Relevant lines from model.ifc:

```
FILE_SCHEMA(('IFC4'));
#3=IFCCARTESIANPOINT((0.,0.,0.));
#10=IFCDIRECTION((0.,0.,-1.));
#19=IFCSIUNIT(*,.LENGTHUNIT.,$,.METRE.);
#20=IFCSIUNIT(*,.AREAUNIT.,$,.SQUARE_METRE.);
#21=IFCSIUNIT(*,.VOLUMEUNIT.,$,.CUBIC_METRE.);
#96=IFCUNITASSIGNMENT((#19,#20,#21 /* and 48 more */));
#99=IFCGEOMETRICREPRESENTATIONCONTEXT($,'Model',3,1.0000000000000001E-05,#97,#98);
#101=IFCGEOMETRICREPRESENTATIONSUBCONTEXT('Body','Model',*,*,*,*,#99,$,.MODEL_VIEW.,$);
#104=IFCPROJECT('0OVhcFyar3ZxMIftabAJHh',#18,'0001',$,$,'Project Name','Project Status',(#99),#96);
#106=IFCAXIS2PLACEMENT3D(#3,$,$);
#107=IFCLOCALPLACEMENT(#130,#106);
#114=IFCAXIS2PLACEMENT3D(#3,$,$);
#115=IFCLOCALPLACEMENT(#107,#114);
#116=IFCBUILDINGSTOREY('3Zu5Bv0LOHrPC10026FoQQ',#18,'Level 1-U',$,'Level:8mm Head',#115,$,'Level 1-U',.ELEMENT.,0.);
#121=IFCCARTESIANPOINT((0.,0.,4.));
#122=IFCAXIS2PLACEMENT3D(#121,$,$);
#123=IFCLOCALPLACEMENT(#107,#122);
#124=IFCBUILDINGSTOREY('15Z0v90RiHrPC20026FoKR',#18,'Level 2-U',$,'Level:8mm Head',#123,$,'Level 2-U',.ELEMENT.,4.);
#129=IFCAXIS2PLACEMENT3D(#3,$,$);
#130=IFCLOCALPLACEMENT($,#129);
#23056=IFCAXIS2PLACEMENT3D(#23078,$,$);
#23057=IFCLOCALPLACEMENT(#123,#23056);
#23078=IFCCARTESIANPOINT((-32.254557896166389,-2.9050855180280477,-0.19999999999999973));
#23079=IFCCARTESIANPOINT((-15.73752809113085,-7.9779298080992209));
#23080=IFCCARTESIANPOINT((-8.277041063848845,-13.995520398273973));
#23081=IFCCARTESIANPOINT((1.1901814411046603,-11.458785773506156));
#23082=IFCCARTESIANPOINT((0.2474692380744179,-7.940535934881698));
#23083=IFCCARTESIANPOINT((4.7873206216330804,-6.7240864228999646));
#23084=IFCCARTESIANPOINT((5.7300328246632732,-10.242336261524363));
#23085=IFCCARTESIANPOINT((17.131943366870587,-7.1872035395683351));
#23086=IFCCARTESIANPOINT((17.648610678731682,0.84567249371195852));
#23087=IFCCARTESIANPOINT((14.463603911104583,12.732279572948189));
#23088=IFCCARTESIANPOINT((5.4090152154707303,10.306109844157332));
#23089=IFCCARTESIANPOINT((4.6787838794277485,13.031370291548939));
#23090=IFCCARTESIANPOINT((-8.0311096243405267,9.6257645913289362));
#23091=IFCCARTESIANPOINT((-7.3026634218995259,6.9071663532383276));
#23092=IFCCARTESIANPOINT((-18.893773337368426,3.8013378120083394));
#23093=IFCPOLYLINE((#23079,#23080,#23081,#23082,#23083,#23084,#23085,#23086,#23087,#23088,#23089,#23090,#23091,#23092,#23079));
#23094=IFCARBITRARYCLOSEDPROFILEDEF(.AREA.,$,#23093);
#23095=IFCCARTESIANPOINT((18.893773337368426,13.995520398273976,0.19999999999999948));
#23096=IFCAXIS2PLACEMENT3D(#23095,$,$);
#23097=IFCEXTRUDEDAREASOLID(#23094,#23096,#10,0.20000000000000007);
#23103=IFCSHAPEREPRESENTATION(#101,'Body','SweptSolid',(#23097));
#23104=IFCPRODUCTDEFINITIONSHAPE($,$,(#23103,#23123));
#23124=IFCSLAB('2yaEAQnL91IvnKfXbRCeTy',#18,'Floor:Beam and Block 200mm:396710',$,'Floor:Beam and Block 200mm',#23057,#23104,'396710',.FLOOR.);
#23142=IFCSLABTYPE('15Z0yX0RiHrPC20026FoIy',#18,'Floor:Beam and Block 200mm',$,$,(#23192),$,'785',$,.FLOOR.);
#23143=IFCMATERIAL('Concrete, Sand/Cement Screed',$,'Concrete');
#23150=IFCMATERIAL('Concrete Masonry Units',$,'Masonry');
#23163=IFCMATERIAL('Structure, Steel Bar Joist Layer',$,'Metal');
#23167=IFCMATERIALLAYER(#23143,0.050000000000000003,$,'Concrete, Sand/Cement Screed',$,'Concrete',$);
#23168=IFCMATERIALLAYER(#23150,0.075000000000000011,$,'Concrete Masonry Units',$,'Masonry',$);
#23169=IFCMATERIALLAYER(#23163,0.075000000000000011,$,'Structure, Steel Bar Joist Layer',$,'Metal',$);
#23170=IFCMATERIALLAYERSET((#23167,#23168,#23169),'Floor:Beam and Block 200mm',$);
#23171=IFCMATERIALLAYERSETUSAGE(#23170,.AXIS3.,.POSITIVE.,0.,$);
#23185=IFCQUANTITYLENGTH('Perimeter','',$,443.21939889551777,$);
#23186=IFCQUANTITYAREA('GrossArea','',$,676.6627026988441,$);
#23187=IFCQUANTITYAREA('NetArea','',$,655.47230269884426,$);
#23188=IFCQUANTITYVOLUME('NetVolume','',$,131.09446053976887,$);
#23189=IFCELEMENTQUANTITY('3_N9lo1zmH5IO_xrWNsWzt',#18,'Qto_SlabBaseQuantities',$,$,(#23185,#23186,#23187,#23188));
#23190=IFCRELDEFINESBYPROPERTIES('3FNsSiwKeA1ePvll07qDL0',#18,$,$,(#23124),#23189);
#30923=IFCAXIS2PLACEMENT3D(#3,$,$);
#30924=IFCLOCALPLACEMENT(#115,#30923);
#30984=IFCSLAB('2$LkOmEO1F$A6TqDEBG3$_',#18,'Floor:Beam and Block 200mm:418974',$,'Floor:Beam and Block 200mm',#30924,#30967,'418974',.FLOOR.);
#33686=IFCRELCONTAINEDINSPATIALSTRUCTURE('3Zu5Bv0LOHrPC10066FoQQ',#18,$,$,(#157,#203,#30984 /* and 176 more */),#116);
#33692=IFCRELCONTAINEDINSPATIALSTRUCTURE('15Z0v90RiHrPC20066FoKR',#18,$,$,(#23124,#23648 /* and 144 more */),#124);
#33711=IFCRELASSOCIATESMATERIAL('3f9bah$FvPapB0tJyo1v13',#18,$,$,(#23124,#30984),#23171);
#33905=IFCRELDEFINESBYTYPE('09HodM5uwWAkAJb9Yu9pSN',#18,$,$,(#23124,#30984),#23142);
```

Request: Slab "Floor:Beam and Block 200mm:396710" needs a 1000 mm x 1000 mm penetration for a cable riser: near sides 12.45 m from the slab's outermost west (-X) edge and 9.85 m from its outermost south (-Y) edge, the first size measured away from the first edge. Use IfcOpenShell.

```python
import numpy as np
import ifcopenshell
import ifcopenshell.api.feature
import ifcopenshell.api.geometry
import ifcopenshell.api.pset
import ifcopenshell.api.root
import ifcopenshell.geom
import ifcopenshell.util.element
import ifcopenshell.util.placement
import ifcopenshell.util.representation
import ifcopenshell.util.shape
import ifcopenshell.util.unit

model = ifcopenshell.open("model.ifc")
unit_scale = ifcopenshell.util.unit.calculate_unit_scale(model)
area_scale = ifcopenshell.util.unit.calculate_unit_scale(model, "AREAUNIT")
volume_scale = ifcopenshell.util.unit.calculate_unit_scale(model, "VOLUMEUNIT")
settings = ifcopenshell.geom.settings()


def volume(element):
    """Net volume in cubic metres, openings subtracted."""
    shape = ifcopenshell.geom.create_shape(settings, element)
    return ifcopenshell.util.shape.get_volume(shape.geometry)


slab = model.by_id(23124)
before = volume(slab)

# Extent in the slab's own axes, in metres. The edges named are its -X and -Y sides.
slab_shape = ifcopenshell.geom.create_shape(settings, slab)
vertices = ifcopenshell.util.shape.get_vertices(slab_shape.geometry)
x_min, y_min, bottom = vertices.min(axis=0)
top = vertices[:, 2].max()

opening = ifcopenshell.api.root.create_entity(model, ifc_class="IfcOpeningElement", name="Cable riser opening", predefined_type="OPENING")
context = ifcopenshell.util.representation.get_context(model, "Model", "Body", "MODEL_VIEW")
width, depth = 1, 1
outline = [(0.0, 0.0), (width, 0.0), (width, depth), (0.0, depth), (0.0, 0.0)]
# Overshoot both faces by 50 mm so the cut is clean.
shape = ifcopenshell.api.geometry.add_slab_representation(
    model, context=context, depth=top - bottom + 0.1, polyline=outline
)
ifcopenshell.api.geometry.assign_representation(model, product=opening, representation=shape)

matrix = ifcopenshell.util.placement.get_local_placement(slab.ObjectPlacement)
matrix[:, 3] = matrix @ np.append(np.array([x_min + 12.45, y_min + 9.85, bottom - 0.05]) / unit_scale, 1.0)
ifcopenshell.api.geometry.edit_object_placement(model, product=opening, matrix=matrix, is_si=False)
ifcopenshell.api.feature.add_feature(model, feature=opening, element=slab)

after = volume(slab)

# Update the slab's stored quantities.
qto = model.by_id(ifcopenshell.util.element.get_pset(slab, "Qto_SlabBaseQuantities", should_inherit=False)["id"])
ifcopenshell.api.pset.edit_qto(model, qto=qto, properties={
    "NetArea": after / (top - bottom) / area_scale,
    "NetVolume": after / volume_scale,
})

print(f"slab volume {before:.3f} -> {after:.3f} m3")

model.write("model-out.ifc")
```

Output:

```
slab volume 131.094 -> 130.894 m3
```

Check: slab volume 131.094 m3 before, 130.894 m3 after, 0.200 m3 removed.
